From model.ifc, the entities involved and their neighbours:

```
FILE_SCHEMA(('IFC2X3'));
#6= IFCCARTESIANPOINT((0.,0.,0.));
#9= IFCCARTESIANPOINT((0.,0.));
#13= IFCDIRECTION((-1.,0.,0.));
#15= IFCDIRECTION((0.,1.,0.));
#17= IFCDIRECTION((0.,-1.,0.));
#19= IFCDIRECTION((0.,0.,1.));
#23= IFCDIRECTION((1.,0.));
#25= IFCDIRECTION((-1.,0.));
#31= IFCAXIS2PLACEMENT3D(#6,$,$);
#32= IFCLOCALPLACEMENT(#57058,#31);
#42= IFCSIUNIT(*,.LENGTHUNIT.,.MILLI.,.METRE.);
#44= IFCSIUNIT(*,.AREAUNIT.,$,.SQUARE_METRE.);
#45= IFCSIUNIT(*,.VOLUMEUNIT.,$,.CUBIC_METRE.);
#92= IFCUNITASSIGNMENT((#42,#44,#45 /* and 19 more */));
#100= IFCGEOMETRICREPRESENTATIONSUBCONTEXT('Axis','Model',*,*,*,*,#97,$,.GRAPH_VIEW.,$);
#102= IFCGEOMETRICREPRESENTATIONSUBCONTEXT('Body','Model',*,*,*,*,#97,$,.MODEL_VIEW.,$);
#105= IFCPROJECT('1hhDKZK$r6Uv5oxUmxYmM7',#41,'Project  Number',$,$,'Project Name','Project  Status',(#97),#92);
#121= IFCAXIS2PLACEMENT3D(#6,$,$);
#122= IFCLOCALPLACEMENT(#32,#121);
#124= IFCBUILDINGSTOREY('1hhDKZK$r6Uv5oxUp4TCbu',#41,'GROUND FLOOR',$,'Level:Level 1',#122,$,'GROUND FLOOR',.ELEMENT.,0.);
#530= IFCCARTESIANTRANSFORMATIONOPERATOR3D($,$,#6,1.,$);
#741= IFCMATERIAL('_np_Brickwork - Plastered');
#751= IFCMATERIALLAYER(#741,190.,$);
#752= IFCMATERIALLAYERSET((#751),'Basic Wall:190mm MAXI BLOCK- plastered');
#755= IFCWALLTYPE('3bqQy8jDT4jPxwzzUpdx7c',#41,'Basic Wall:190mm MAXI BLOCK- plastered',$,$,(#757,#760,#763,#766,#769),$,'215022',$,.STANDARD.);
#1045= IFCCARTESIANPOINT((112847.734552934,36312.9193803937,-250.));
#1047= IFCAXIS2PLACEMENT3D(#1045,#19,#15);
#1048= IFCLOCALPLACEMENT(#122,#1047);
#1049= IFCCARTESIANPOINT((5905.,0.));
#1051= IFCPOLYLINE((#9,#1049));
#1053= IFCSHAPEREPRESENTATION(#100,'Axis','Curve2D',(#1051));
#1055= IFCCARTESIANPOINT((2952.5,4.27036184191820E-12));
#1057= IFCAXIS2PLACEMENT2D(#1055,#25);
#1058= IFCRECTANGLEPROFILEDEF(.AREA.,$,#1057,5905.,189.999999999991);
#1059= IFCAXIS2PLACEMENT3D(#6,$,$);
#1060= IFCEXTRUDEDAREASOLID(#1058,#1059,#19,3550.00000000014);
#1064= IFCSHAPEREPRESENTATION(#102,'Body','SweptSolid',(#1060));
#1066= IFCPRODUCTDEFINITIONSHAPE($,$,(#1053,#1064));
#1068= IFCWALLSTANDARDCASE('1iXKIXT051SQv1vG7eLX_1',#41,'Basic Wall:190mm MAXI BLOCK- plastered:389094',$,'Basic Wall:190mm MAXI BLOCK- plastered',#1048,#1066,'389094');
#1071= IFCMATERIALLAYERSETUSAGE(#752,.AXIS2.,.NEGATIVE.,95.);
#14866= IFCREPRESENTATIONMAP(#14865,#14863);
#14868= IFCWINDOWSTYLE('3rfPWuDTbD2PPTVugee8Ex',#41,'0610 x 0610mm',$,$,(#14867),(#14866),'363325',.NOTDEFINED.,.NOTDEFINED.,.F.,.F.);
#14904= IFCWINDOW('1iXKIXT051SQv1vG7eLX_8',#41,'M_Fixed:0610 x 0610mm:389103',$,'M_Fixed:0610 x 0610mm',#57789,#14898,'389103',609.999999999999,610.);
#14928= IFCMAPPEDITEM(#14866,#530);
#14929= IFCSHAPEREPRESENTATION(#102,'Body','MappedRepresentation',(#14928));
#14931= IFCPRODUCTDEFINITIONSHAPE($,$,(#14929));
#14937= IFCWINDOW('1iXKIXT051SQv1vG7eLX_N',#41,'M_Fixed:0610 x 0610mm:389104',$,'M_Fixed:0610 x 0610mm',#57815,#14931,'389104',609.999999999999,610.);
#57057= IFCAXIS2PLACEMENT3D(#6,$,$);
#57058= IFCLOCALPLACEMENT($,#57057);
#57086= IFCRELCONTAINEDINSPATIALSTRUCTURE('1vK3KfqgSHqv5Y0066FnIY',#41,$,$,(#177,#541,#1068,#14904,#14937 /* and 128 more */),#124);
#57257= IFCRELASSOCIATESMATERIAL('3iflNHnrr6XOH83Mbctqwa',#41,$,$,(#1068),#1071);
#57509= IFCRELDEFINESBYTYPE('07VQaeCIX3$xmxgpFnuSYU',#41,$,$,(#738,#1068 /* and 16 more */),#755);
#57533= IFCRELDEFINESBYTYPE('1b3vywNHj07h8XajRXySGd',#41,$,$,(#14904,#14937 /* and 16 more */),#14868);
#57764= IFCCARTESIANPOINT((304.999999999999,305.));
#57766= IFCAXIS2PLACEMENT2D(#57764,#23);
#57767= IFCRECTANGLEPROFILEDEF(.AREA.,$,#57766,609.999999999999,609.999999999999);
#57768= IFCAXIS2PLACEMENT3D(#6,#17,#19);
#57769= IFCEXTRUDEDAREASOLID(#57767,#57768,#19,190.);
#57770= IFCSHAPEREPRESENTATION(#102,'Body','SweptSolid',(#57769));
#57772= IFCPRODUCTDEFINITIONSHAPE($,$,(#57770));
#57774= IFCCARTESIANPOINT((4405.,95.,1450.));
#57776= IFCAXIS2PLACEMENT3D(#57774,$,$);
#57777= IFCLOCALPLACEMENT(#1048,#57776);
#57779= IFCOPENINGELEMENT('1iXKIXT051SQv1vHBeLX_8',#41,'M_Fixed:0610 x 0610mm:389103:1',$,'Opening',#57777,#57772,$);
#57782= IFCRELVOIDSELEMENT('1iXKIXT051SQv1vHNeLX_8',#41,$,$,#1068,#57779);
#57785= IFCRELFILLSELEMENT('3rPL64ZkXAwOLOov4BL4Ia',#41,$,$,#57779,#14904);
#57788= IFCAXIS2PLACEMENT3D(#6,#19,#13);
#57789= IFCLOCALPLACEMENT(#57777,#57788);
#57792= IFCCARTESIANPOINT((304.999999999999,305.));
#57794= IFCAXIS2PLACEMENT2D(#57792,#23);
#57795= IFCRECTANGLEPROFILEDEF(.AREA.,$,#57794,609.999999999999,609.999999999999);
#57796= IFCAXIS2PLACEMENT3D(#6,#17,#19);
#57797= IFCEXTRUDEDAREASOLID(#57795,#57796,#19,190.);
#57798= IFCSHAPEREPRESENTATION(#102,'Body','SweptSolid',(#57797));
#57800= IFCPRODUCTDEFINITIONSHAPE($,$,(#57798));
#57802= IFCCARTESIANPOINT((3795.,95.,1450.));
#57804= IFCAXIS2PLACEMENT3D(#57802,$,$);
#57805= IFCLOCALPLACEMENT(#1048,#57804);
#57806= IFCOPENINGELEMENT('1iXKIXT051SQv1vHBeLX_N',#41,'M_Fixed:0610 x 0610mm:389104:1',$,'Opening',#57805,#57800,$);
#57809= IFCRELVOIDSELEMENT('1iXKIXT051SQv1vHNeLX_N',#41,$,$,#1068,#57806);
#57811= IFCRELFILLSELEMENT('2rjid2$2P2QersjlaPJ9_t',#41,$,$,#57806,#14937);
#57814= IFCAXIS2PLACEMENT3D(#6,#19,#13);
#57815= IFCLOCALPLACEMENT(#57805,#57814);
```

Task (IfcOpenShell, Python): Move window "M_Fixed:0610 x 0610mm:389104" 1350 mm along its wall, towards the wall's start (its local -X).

```python
import ifcopenshell
import ifcopenshell.api.geometry
import ifcopenshell.util.placement

model = ifcopenshell.open("model.ifc")

window = model.by_guid("1iXKIXT051SQv1vG7eLX_N")
opening = window.FillsVoids[0].RelatingOpeningElement
wall = opening.VoidsElements[0].RelatingBuildingElement

wall_matrix = ifcopenshell.util.placement.get_local_placement(wall.ObjectPlacement)
shift = wall_matrix[:3, 0] * -1350.0
before = ifcopenshell.util.placement.get_local_placement(window.ObjectPlacement)[:3, 3].copy()

# The window is placed relative to its opening, so it follows when the opening moves.
matrix = ifcopenshell.util.placement.get_local_placement(opening.ObjectPlacement)
matrix[:3, 3] += shift
ifcopenshell.api.geometry.edit_object_placement(
    model, product=opening, matrix=matrix, is_si=False, should_transform_children=True
)

after = ifcopenshell.util.placement.get_local_placement(window.ObjectPlacement)[:3, 3]
print("window moved by", (after - before).round(3) + 0.0)

model.write("model_v2.ifc")
```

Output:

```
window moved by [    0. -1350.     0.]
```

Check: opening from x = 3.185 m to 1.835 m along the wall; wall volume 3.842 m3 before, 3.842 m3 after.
